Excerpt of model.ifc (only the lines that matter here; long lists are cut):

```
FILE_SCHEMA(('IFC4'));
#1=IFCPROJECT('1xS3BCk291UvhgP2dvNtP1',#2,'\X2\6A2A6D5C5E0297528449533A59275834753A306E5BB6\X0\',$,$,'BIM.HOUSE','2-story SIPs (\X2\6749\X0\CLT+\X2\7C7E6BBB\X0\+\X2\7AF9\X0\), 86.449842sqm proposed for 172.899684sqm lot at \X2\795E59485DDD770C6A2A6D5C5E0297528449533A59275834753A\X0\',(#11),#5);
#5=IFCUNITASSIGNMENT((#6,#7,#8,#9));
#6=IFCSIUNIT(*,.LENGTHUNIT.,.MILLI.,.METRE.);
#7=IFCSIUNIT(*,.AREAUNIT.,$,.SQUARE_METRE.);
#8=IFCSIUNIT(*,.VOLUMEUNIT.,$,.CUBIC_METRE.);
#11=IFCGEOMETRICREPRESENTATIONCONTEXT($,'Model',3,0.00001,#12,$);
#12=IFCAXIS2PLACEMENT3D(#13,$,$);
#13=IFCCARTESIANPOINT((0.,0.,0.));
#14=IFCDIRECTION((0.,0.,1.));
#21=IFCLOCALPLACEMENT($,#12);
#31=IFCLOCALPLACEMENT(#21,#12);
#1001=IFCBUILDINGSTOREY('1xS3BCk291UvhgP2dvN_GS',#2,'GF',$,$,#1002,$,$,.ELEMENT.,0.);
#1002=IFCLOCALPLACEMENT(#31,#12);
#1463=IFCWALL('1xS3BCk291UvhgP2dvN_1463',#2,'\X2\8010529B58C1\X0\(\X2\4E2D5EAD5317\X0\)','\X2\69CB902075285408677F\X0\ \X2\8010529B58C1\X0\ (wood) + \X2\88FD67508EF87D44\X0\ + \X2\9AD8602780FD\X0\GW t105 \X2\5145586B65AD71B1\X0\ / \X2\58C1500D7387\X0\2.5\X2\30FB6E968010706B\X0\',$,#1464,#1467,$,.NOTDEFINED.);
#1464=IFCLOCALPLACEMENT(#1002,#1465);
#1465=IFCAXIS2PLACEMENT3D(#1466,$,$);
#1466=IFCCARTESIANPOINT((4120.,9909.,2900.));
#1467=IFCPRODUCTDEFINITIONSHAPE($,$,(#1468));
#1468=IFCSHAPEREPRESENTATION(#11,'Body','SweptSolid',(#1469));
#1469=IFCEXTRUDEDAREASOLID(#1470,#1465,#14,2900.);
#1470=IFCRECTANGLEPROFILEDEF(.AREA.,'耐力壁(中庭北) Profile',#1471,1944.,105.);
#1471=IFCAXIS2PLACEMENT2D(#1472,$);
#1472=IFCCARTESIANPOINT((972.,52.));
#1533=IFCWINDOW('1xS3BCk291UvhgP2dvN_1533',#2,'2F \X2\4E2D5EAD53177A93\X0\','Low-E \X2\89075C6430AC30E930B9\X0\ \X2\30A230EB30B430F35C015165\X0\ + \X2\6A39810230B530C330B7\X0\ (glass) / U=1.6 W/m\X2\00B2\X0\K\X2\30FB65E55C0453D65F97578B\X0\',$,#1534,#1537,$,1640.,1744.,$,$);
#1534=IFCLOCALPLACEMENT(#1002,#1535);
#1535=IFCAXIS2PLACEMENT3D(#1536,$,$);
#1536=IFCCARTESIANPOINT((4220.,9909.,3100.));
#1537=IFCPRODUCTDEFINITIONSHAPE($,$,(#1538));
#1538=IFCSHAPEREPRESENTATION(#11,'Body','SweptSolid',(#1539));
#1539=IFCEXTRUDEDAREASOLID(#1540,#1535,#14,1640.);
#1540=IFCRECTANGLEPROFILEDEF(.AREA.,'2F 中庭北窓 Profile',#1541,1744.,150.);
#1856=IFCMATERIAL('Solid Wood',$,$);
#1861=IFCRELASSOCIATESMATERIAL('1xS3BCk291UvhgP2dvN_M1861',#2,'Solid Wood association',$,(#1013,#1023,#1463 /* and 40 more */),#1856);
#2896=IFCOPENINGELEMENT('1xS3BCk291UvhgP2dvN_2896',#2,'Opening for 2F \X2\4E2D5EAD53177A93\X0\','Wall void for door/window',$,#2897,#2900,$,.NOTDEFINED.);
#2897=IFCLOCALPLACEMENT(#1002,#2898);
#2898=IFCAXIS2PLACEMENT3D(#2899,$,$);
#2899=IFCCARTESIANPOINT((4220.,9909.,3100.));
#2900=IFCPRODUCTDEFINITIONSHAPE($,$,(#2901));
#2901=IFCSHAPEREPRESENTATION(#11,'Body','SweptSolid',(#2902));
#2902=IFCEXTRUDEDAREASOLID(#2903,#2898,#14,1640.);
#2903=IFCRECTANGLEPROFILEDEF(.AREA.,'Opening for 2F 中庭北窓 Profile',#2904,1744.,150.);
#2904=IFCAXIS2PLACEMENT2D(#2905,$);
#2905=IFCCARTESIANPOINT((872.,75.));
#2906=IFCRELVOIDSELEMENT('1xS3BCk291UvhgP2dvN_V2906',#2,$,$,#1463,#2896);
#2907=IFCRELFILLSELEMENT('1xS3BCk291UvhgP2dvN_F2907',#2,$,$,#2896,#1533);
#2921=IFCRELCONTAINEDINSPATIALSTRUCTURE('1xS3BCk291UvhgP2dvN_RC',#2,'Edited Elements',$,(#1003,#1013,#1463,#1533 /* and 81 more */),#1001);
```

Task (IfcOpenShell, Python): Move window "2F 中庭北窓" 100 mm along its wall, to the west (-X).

```python
import ifcopenshell
import ifcopenshell.api.geometry
import ifcopenshell.util.placement
import ifcopenshell.util.unit

model = ifcopenshell.open("model.ifc")
unit_scale = ifcopenshell.util.unit.calculate_unit_scale(model)

window = model.by_guid("1xS3BCk291UvhgP2dvN_1533")
opening = window.FillsVoids[0].RelatingOpeningElement
wall = opening.VoidsElements[0].RelatingBuildingElement

wall_matrix = ifcopenshell.util.placement.get_local_placement(wall.ObjectPlacement)
shift = wall_matrix[:3, 0] * -0.1 / unit_scale
before = ifcopenshell.util.placement.get_local_placement(window.ObjectPlacement)[:3, 3].copy()

# The window is not placed relative to its opening, so move both.
for product in (opening, window):
    matrix = ifcopenshell.util.placement.get_local_placement(product.ObjectPlacement)
    matrix[:3, 3] += shift
    ifcopenshell.api.geometry.edit_object_placement(model, product=product, matrix=matrix, is_si=False)

after = ifcopenshell.util.placement.get_local_placement(window.ObjectPlacement)[:3, 3]
print("window moved by", (after - before).round(3) + 0.0)

model.write("model_v2.ifc")
```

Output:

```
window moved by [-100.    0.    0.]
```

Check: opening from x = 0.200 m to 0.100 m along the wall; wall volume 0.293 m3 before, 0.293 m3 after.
